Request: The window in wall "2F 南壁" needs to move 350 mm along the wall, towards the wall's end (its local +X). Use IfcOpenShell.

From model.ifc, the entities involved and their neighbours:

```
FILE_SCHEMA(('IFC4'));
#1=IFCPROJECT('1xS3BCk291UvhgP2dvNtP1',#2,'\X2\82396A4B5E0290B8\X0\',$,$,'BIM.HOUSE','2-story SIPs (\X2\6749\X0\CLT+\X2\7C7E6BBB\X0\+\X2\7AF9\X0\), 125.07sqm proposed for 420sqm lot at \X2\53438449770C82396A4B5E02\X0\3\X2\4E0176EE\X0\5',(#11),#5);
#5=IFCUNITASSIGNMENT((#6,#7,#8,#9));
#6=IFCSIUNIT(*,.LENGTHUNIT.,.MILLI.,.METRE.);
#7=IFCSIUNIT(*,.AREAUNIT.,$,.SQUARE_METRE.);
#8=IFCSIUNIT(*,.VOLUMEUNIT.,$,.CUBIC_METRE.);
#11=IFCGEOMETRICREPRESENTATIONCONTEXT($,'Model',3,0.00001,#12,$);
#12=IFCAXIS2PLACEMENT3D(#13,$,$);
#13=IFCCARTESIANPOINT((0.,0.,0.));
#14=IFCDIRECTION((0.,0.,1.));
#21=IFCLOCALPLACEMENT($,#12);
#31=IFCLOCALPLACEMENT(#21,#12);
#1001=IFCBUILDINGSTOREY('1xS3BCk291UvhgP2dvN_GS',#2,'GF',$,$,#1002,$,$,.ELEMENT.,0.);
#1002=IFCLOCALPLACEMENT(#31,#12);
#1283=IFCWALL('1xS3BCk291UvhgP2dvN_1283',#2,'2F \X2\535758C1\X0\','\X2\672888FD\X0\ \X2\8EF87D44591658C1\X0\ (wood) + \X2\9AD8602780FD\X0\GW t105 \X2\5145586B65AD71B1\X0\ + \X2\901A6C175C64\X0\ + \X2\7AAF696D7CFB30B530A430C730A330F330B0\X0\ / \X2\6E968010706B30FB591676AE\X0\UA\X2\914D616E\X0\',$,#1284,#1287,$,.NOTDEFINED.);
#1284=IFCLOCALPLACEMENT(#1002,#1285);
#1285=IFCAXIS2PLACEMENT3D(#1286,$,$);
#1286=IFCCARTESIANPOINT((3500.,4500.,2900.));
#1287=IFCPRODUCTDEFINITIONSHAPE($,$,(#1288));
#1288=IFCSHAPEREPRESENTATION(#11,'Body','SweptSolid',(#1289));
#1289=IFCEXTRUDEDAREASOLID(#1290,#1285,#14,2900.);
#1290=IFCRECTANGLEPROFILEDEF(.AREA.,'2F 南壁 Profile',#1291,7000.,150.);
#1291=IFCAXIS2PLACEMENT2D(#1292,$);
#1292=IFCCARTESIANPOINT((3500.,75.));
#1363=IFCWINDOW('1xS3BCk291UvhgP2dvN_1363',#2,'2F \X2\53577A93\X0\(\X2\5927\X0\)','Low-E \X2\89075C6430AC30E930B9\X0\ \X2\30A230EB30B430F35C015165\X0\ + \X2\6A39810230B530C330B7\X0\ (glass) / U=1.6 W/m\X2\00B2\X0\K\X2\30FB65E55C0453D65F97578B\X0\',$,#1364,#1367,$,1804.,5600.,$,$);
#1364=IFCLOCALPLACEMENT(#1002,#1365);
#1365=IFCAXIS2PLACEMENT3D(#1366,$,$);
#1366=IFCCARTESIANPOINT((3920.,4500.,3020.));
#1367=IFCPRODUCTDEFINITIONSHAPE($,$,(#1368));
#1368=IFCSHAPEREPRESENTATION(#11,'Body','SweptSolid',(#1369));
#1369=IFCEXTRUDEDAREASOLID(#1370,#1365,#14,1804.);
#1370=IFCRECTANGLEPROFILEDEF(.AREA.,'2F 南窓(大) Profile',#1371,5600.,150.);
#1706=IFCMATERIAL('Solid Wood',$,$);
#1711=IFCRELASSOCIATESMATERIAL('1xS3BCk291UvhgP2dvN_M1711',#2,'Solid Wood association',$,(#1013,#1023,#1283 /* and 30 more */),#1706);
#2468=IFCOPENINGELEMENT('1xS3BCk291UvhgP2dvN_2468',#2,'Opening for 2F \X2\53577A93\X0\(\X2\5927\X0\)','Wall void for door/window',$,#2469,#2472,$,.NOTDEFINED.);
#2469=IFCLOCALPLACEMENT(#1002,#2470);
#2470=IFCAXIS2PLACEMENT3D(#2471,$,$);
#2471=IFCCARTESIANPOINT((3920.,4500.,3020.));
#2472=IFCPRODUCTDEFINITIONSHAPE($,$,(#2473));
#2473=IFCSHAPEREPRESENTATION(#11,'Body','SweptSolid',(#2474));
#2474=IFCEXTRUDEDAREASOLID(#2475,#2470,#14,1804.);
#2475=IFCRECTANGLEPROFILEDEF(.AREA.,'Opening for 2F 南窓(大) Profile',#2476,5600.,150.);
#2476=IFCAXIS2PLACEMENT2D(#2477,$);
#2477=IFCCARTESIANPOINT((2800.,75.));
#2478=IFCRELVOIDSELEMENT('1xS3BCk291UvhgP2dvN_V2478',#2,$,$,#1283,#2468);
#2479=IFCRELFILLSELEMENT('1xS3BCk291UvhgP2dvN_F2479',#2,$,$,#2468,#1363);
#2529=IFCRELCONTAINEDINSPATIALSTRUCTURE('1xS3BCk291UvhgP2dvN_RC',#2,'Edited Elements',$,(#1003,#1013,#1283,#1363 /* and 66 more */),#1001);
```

```python
import ifcopenshell
import ifcopenshell.api.geometry
import ifcopenshell.util.placement
import ifcopenshell.util.unit

model = ifcopenshell.open("model.ifc")
unit_scale = ifcopenshell.util.unit.calculate_unit_scale(model)

window = model.by_guid("1xS3BCk291UvhgP2dvN_1363")
opening = window.FillsVoids[0].RelatingOpeningElement
wall = opening.VoidsElements[0].RelatingBuildingElement

wall_matrix = ifcopenshell.util.placement.get_local_placement(wall.ObjectPlacement)
shift = wall_matrix[:3, 0] * 0.35 / unit_scale
before = ifcopenshell.util.placement.get_local_placement(window.ObjectPlacement)[:3, 3].copy()

# The window is not placed relative to its opening, so move both.
for product in (opening, window):
    matrix = ifcopenshell.util.placement.get_local_placement(product.ObjectPlacement)
    matrix[:3, 3] += shift
    ifcopenshell.api.geometry.edit_object_placement(model, product=product, matrix=matrix, is_si=False)

after = ifcopenshell.util.placement.get_local_placement(window.ObjectPlacement)[:3, 3]
print("window moved by", (after - before).round(3) + 0.0)

model.write("model_rev.ifc")
```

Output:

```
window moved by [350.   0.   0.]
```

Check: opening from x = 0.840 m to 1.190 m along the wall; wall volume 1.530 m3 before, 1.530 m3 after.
